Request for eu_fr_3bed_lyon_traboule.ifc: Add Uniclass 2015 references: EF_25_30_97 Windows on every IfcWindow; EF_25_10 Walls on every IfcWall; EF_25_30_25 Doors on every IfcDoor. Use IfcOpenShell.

First a look at what the model holds.

```python
import ifcopenshell

model = ifcopenshell.open("eu_fr_3bed_lyon_traboule.ifc")
print(model.schema)
print("classifications:", [c.Name for c in model.by_type("IfcClassification")])
for ifc_class in ("IfcDoor", "IfcRoof", "IfcStair", "IfcWall", "IfcWindow"):
    print(ifc_class, len(model.by_type(ifc_class)))
```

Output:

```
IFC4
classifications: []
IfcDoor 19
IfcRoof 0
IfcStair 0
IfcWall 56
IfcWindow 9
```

```python
import ifcopenshell
import ifcopenshell.api.classification

model = ifcopenshell.open("eu_fr_3bed_lyon_traboule.ifc")

system = ifcopenshell.api.classification.add_classification(model, classification="Uniclass 2015")

codes = {
    "IfcWindow": ("EF_25_30_97", "Windows"),
    "IfcWall": ("EF_25_10", "Walls"),
    "IfcDoor": ("EF_25_30_25", "Doors"),
}
for ifc_class, (code, name) in codes.items():
    products = model.by_type(ifc_class)
    ifcopenshell.api.classification.add_reference(
        model, products=products, classification=system, identification=code, name=name
    )
    print(code, len(products))

model.write("eu_fr_3bed_lyon_traboule_v2.ifc")
```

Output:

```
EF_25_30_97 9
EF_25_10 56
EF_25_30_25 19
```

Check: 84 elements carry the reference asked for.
